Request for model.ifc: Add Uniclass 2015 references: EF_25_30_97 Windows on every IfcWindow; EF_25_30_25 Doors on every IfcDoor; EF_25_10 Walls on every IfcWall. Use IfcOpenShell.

First a look at what the model holds.

```python
import ifcopenshell

model = ifcopenshell.open("model.ifc")
print(model.schema)
print("classifications:", [c.Name for c in model.by_type("IfcClassification")])
for ifc_class in ("IfcDoor", "IfcRoof", "IfcStair", "IfcWall", "IfcWindow"):
    print(ifc_class, len(model.by_type(ifc_class)))
```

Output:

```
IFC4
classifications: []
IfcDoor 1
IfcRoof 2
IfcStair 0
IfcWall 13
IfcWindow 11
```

```python
import ifcopenshell
import ifcopenshell.api.classification

model = ifcopenshell.open("model.ifc")

system = ifcopenshell.api.classification.add_classification(model, classification="Uniclass 2015")

codes = {
    "IfcWindow": ("EF_25_30_97", "Windows"),
    "IfcDoor": ("EF_25_30_25", "Doors"),
    "IfcWall": ("EF_25_10", "Walls"),
}
for ifc_class, (code, name) in codes.items():
    products = model.by_type(ifc_class)
    ifcopenshell.api.classification.add_reference(
        model, products=products, classification=system, identification=code, name=name
    )
    print(code, len(products))

model.write("model_edited.ifc")
```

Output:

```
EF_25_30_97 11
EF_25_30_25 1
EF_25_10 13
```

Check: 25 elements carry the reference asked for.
